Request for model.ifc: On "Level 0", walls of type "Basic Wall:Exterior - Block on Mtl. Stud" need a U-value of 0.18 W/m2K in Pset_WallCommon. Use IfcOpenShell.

First a look at what the model holds.

```python
import ifcopenshell
import ifcopenshell.util.element

model = ifcopenshell.open("model.ifc")
print(model.schema)
storey = next(s for s in model.by_type("IfcBuildingStorey") if s.Name == "Level 0")
walls = [e for e in ifcopenshell.util.element.get_decomposition(storey) if e.is_a("IfcWall")]
seen = {}
for e in walls:
    element_type = ifcopenshell.util.element.get_type(e)
    key = (element_type.Name if element_type != e and element_type else None, ifcopenshell.util.element.get_pset(e, "Pset_WallCommon", "ThermalTransmittance"))
    seen[key] = seen.get(key, 0) + 1
for (name, value), count in sorted(seen.items(), key=str):
    print(count, "x", name, "|", value)
```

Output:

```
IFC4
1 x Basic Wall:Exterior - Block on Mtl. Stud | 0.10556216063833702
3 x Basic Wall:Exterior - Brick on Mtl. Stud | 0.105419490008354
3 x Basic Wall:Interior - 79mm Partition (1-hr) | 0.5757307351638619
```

```python
import ifcopenshell
import ifcopenshell.api.pset
import ifcopenshell.util.element

model = ifcopenshell.open("model.ifc")

storey = next(s for s in model.by_type("IfcBuildingStorey") if s.Name == "Level 0")
walls = [e for e in ifcopenshell.util.element.get_decomposition(storey) if e.is_a("IfcWall")]

count = 0
for e in walls:
    element_type = ifcopenshell.util.element.get_type(e)
    if element_type in (None, e) or element_type.Name != "Basic Wall:Exterior - Block on Mtl. Stud":
        continue
    # add_pset returns the element's existing set when there is one.
    pset = ifcopenshell.api.pset.add_pset(model, product=e, name="Pset_WallCommon")
    ifcopenshell.api.pset.edit_pset(model, pset=pset, properties={"ThermalTransmittance": 0.18})
    count += 1

print(count, "walls updated")

model.write("model_edited.ifc")
```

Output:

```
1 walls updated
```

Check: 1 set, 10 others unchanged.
